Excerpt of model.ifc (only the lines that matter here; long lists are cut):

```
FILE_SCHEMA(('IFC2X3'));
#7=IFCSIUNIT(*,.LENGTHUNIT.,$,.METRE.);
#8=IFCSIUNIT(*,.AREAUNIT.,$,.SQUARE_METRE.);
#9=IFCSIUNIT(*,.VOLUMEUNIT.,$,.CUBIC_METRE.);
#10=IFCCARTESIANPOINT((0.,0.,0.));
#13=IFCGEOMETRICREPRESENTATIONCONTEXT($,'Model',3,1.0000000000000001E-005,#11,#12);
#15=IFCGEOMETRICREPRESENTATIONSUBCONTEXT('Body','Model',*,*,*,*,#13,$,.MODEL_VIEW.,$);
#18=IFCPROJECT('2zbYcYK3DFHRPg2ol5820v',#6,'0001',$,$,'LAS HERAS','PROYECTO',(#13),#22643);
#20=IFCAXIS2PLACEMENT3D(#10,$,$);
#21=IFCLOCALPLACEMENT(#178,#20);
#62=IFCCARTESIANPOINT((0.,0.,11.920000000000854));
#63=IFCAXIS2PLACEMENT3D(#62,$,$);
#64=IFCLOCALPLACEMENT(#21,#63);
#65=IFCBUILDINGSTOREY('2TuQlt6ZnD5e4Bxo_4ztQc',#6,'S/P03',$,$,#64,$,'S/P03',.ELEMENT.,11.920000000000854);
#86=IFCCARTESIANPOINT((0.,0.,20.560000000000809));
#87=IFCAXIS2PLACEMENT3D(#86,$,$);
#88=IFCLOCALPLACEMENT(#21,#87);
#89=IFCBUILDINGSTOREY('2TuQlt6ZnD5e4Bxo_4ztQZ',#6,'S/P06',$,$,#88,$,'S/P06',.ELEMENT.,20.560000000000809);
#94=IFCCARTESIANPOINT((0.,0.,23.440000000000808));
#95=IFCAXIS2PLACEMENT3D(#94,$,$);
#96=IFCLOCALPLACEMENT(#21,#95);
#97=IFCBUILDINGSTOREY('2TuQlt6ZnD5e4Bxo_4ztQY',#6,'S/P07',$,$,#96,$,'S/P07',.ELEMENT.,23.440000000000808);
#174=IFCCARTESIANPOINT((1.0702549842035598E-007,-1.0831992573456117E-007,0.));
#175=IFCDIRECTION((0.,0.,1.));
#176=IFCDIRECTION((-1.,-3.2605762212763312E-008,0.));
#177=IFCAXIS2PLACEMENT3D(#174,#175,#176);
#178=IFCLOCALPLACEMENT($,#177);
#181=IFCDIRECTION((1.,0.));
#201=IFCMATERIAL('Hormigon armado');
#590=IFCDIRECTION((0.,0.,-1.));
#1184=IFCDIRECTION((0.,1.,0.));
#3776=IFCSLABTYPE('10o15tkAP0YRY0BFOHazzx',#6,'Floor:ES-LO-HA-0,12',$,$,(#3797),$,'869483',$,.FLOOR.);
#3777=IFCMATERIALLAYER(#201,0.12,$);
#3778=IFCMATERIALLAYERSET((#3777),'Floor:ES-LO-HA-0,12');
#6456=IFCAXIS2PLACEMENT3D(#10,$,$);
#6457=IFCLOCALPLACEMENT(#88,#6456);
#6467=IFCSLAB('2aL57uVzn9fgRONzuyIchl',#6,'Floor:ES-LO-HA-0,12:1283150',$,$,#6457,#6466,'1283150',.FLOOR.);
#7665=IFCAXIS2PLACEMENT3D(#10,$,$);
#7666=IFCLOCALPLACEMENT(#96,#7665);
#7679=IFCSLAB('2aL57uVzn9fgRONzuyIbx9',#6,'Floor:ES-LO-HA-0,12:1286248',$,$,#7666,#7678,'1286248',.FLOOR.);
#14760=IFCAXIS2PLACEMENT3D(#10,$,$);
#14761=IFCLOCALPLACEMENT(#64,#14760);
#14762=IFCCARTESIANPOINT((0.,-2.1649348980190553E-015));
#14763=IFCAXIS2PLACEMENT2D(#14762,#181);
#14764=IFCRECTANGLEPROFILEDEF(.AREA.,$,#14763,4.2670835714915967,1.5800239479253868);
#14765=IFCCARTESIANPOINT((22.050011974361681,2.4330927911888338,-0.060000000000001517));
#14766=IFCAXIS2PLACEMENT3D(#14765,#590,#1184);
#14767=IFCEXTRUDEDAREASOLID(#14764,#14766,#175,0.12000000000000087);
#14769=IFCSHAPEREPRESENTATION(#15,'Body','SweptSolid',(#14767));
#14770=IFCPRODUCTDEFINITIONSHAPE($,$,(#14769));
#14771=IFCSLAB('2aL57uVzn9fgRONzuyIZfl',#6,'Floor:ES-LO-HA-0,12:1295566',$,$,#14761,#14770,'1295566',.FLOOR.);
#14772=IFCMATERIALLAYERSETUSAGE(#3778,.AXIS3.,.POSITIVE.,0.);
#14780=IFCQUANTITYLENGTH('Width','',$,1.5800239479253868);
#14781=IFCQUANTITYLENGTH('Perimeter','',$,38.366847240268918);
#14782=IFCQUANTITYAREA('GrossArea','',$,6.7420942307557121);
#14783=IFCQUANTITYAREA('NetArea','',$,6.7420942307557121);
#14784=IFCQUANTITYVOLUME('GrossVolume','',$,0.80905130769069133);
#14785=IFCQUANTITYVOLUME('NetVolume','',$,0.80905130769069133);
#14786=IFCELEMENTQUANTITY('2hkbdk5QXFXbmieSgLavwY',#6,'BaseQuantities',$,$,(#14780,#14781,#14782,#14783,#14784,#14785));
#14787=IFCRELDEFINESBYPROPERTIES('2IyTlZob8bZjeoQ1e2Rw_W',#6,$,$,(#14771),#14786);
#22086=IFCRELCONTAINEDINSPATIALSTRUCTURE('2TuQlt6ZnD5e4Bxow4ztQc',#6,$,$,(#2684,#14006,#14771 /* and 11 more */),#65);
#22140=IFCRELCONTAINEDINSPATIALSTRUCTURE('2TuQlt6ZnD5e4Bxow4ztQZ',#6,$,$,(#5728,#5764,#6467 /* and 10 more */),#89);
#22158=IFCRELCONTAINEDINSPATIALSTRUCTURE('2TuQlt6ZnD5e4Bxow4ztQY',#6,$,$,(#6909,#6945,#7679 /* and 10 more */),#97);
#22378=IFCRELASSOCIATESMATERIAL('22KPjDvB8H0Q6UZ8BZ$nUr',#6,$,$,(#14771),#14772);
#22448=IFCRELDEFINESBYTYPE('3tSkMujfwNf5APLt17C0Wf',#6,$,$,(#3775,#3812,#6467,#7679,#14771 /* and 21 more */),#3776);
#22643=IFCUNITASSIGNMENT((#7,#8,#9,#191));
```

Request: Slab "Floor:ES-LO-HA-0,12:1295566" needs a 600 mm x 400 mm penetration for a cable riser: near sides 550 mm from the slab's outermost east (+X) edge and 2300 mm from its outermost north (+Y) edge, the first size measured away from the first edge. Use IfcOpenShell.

```python
import numpy as np
import ifcopenshell
import ifcopenshell.api.feature
import ifcopenshell.api.geometry
import ifcopenshell.api.pset
import ifcopenshell.api.root
import ifcopenshell.geom
import ifcopenshell.util.element
import ifcopenshell.util.placement
import ifcopenshell.util.representation
import ifcopenshell.util.shape
import ifcopenshell.util.unit

model = ifcopenshell.open("model.ifc")
unit_scale = ifcopenshell.util.unit.calculate_unit_scale(model)
area_scale = ifcopenshell.util.unit.calculate_unit_scale(model, "AREAUNIT")
volume_scale = ifcopenshell.util.unit.calculate_unit_scale(model, "VOLUMEUNIT")
settings = ifcopenshell.geom.settings()


def volume(element):
    """Net volume in cubic metres, openings subtracted."""
    shape = ifcopenshell.geom.create_shape(settings, element)
    return ifcopenshell.util.shape.get_volume(shape.geometry)


slab = model.by_guid("2aL57uVzn9fgRONzuyIZfl")
before = volume(slab)

# Extent in the slab's own axes, in metres. The edges named are its -X and -Y sides.
slab_shape = ifcopenshell.geom.create_shape(settings, slab)
vertices = ifcopenshell.util.shape.get_vertices(slab_shape.geometry)
x_min, y_min, bottom = vertices.min(axis=0)
top = vertices[:, 2].max()

opening = ifcopenshell.api.root.create_entity(model, ifc_class="IfcOpeningElement", name="Cable riser opening")
context = ifcopenshell.util.representation.get_context(model, "Model", "Body", "MODEL_VIEW")
width, depth = 0.6, 0.4
outline = [(0.0, 0.0), (width, 0.0), (width, depth), (0.0, depth), (0.0, 0.0)]
# Overshoot both faces by 50 mm so the cut is clean.
shape = ifcopenshell.api.geometry.add_slab_representation(
    model, context=context, depth=top - bottom + 0.1, polyline=outline
)
ifcopenshell.api.geometry.assign_representation(model, product=opening, representation=shape)

matrix = ifcopenshell.util.placement.get_local_placement(slab.ObjectPlacement)
matrix[:, 3] = matrix @ np.append(np.array([x_min + 0.55, y_min + 2.3, bottom - 0.05]) / unit_scale, 1.0)
ifcopenshell.api.geometry.edit_object_placement(model, product=opening, matrix=matrix, is_si=False)
ifcopenshell.api.feature.add_feature(model, feature=opening, element=slab)

after = volume(slab)

# Update the slab's stored quantities.
qto = model.by_id(ifcopenshell.util.element.get_pset(slab, "BaseQuantities", should_inherit=False)["id"])
ifcopenshell.api.pset.edit_qto(model, qto=qto, properties={
    "NetArea": after / (top - bottom) / area_scale,
    "NetVolume": after / volume_scale,
})

print(f"slab volume {before:.3f} -> {after:.3f} m3")

model.write("model-out.ifc")
```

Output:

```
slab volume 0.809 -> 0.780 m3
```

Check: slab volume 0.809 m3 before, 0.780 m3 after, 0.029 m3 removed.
